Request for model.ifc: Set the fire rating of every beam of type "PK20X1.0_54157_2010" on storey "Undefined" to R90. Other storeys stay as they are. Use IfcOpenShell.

First a look at what the model holds.

```python
import ifcopenshell
import ifcopenshell.util.element

model = ifcopenshell.open("model.ifc")
print(model.schema)
storey = next(s for s in model.by_type("IfcBuildingStorey") if s.Name == "Undefined")
beams = [e for e in ifcopenshell.util.element.get_decomposition(storey) if e.is_a("IfcBeam")]
seen = {}
for e in beams:
    element_type = ifcopenshell.util.element.get_type(e)
    key = (element_type.Name if element_type != e and element_type else None, ifcopenshell.util.element.get_pset(e, "Pset_BeamCommon", "FireRating"))
    seen[key] = seen.get(key, 0) + 1
for (name, value), count in sorted(seen.items(), key=str):
    print(count, "x", name, "|", value)
```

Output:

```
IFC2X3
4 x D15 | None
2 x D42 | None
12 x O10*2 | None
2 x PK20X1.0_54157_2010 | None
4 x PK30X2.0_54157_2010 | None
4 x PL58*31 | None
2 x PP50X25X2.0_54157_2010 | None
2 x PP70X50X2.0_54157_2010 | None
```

```python
import ifcopenshell
import ifcopenshell.api.pset
import ifcopenshell.util.element

model = ifcopenshell.open("model.ifc")

storey = next(s for s in model.by_type("IfcBuildingStorey") if s.Name == "Undefined")
beams = [e for e in ifcopenshell.util.element.get_decomposition(storey) if e.is_a("IfcBeam")]

count = 0
for e in beams:
    element_type = ifcopenshell.util.element.get_type(e)
    if element_type in (None, e) or element_type.Name != "PK20X1.0_54157_2010":
        continue
    found = ifcopenshell.util.element.get_pset(e, "Pset_BeamCommon", should_inherit=False)
    if found:
        pset = model.by_id(found["id"])
        if len(ifcopenshell.util.element.get_elements_by_pset(pset)) > 1:
            pset = ifcopenshell.api.pset.unshare_pset(model, products=[e], pset=pset)[0]
    else:
        pset = ifcopenshell.api.pset.add_pset(model, product=e, name="Pset_BeamCommon")
    ifcopenshell.api.pset.edit_pset(model, pset=pset, properties={"FireRating": "R90"})
    count += 1

print(count, "beams updated")

model.write("model_updated.ifc")
```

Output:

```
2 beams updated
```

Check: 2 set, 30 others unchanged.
